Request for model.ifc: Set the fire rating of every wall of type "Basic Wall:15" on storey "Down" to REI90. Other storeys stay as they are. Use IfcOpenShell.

First a look at what the model holds.

```python
import ifcopenshell
import ifcopenshell.util.element

model = ifcopenshell.open("model.ifc")
print(model.schema)
storey = next(s for s in model.by_type("IfcBuildingStorey") if s.Name == "Down")
walls = [e for e in ifcopenshell.util.element.get_decomposition(storey) if e.is_a("IfcWall")]
seen = {}
for e in walls:
    element_type = ifcopenshell.util.element.get_type(e)
    key = (element_type.Name if element_type != e and element_type else None, ifcopenshell.util.element.get_pset(e, "Pset_WallCommon", "FireRating"))
    seen[key] = seen.get(key, 0) + 1
for (name, value), count in sorted(seen.items(), key=str):
    print(count, "x", name, "|", value)
```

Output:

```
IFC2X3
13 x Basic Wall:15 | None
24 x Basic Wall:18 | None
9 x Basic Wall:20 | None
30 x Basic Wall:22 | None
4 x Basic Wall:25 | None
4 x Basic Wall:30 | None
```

```python
import ifcopenshell
import ifcopenshell.api.pset
import ifcopenshell.util.element

model = ifcopenshell.open("model.ifc")

storey = next(s for s in model.by_type("IfcBuildingStorey") if s.Name == "Down")
walls = [e for e in ifcopenshell.util.element.get_decomposition(storey) if e.is_a("IfcWall")]

count = 0
for e in walls:
    element_type = ifcopenshell.util.element.get_type(e)
    if element_type in (None, e) or element_type.Name != "Basic Wall:15":
        continue
    # add_pset returns the element's existing set when there is one.
    pset = ifcopenshell.api.pset.add_pset(model, product=e, name="Pset_WallCommon")
    ifcopenshell.api.pset.edit_pset(model, pset=pset, properties={"FireRating": "REI90"})
    count += 1

print(count, "walls updated")

model.write("model_updated.ifc")
```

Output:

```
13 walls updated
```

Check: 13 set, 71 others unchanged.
